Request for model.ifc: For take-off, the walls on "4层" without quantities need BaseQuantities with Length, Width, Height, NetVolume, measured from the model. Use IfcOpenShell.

First a look at what the model holds.

```python
import ifcopenshell
import ifcopenshell.util.element
import ifcopenshell.util.unit

model = ifcopenshell.open("model.ifc")
print(model.schema)
for unit_type in ("LENGTHUNIT", "AREAUNIT", "VOLUMEUNIT"):
    print(unit_type, ifcopenshell.util.unit.calculate_unit_scale(model, unit_type))
storey = next(s for s in model.by_type("IfcBuildingStorey") if s.Name == "4层")
walls = [e for e in ifcopenshell.util.element.get_decomposition(storey) if e.is_a("IfcWall")]
for e in sorted(walls, key=lambda e: e.id()):
    print(e.id(), e.is_a(), e.Name, list(ifcopenshell.util.element.get_psets(e, qtos_only=True)), sep=" | ")
```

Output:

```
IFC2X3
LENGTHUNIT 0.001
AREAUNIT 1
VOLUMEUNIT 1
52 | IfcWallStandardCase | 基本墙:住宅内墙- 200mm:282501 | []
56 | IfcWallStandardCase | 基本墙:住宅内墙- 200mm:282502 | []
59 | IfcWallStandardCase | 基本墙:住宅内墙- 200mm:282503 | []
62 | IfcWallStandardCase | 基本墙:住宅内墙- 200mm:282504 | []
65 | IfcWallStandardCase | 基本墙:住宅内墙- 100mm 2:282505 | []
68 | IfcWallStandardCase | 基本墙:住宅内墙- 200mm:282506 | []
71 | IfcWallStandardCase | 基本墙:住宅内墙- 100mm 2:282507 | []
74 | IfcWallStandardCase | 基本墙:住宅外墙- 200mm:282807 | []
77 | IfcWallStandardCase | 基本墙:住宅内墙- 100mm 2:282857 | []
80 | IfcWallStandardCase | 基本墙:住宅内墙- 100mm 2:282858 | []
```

```python
import ifcopenshell
import ifcopenshell.api.pset
import ifcopenshell.geom
import ifcopenshell.util.element
import ifcopenshell.util.shape
import ifcopenshell.util.unit

model = ifcopenshell.open("model.ifc")
unit_scale = ifcopenshell.util.unit.calculate_unit_scale(model)
volume_scale = ifcopenshell.util.unit.calculate_unit_scale(model, "VOLUMEUNIT")
settings = ifcopenshell.geom.settings()

storey = next(s for s in model.by_type("IfcBuildingStorey") if s.Name == "4层")
walls = [e for e in ifcopenshell.util.element.get_decomposition(storey) if e.is_a("IfcWall")]

for e in sorted(walls, key=lambda e: e.id()):
    if ifcopenshell.util.element.get_psets(e, qtos_only=True, should_inherit=False):
        continue
    # Geometry comes back in metres, in the element's own axes.
    shape = ifcopenshell.geom.create_shape(settings, e)
    values = {
        "Length": ifcopenshell.util.shape.get_x(shape.geometry) / unit_scale,
        "Width": ifcopenshell.util.shape.get_y(shape.geometry) / unit_scale,
        "Height": ifcopenshell.util.shape.get_z(shape.geometry) / unit_scale,
        "NetVolume": ifcopenshell.util.shape.get_volume(shape.geometry) / volume_scale,
    }
    qto = ifcopenshell.api.pset.add_qto(model, product=e, name="BaseQuantities")
    ifcopenshell.api.pset.edit_qto(model, qto=qto, properties=values)
    print(e.id(), {k: round(v, 3) for k, v in values.items()})

model.write("model_v2.ifc")
```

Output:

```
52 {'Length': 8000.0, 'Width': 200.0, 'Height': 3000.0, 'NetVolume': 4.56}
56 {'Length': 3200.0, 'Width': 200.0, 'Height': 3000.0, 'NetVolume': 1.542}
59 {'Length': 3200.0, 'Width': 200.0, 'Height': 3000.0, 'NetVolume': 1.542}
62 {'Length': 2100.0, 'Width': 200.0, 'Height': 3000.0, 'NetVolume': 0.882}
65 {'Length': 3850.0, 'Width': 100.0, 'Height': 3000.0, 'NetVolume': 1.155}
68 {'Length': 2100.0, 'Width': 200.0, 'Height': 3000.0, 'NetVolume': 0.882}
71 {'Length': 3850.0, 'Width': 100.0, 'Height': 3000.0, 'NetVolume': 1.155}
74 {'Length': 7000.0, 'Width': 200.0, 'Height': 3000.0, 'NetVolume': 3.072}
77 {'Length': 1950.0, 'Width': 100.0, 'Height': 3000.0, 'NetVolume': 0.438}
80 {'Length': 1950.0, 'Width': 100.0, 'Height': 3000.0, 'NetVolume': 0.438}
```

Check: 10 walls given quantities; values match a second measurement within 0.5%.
